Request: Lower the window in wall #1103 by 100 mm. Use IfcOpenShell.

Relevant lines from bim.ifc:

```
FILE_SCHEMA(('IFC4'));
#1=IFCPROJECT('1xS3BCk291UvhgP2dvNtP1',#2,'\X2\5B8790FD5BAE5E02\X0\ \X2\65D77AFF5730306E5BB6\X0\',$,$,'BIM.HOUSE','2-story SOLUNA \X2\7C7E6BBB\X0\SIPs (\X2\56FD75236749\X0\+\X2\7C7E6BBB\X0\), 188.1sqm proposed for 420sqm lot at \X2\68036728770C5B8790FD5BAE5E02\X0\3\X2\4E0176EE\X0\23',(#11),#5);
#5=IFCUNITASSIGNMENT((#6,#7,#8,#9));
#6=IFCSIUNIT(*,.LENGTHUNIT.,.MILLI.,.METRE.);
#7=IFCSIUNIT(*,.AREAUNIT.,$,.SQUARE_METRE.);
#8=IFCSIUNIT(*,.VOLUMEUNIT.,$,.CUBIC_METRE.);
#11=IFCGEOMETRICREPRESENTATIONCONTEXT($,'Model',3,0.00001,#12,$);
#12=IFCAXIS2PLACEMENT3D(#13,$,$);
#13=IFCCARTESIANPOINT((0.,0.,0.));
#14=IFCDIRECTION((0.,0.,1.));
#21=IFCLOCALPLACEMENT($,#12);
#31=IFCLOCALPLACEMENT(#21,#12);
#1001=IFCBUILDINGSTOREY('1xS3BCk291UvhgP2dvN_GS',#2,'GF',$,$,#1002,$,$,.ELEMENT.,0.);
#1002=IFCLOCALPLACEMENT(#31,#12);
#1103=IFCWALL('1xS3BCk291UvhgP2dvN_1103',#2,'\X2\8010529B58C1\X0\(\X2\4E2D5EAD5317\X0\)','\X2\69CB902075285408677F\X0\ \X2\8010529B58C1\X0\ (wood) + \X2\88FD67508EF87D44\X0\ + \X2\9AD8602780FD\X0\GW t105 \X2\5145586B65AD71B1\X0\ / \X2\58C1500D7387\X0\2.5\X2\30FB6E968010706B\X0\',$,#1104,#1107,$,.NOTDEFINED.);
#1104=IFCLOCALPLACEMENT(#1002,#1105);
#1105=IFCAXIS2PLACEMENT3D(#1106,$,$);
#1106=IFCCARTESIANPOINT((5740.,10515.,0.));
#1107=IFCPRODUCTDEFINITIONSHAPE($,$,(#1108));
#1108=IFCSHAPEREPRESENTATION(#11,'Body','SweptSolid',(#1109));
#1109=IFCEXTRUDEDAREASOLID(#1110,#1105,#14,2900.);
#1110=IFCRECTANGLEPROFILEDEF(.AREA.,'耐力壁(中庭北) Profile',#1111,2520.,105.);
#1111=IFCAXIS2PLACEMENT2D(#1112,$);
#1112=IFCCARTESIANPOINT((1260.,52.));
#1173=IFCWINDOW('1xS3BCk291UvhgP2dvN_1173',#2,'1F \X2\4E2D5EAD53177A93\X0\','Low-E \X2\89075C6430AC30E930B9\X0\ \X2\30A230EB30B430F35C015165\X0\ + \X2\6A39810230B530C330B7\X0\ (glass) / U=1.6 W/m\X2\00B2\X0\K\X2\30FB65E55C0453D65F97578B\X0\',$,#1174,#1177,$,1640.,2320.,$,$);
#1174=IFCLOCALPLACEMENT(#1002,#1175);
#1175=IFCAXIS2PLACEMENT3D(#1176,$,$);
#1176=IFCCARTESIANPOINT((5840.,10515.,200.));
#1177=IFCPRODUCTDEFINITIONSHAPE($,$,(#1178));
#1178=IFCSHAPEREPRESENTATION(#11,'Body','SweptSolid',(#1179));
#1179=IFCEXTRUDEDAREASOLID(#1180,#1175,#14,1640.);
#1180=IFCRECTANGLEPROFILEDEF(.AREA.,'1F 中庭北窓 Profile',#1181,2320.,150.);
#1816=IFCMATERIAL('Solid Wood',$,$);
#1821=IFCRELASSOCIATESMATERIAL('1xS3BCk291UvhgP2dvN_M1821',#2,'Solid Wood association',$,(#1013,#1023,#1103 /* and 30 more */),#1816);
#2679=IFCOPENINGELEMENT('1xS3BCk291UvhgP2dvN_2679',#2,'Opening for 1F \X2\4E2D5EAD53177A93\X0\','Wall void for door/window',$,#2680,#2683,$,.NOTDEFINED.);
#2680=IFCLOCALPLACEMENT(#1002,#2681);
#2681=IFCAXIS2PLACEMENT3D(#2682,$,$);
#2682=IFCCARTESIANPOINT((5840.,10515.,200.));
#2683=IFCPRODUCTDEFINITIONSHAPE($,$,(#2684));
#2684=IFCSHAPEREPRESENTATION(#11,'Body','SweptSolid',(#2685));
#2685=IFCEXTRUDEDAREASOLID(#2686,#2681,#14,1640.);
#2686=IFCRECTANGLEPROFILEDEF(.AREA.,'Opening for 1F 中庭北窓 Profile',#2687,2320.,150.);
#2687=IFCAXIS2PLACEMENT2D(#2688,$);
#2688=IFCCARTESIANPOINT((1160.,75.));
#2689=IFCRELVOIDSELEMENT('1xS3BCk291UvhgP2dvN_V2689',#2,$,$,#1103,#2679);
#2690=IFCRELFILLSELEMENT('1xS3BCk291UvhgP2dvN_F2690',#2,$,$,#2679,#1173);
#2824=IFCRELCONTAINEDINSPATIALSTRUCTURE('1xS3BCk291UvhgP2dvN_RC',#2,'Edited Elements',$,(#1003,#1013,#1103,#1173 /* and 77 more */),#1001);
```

```python
import numpy as np
import ifcopenshell
import ifcopenshell.api.geometry
import ifcopenshell.util.placement
import ifcopenshell.util.unit

model = ifcopenshell.open("bim.ifc")
unit_scale = ifcopenshell.util.unit.calculate_unit_scale(model)

window = model.by_guid("1xS3BCk291UvhgP2dvN_1173")
opening = window.FillsVoids[0].RelatingOpeningElement
dz = -0.1 / unit_scale

shift = np.array([0.0, 0.0, dz])
# The window is not placed relative to its opening, so move both.
for product in (opening, window):
    matrix = ifcopenshell.util.placement.get_local_placement(product.ObjectPlacement)
    matrix[:3, 3] += shift
    ifcopenshell.api.geometry.edit_object_placement(model, product=product, matrix=matrix, is_si=False)

print(f"moved by {dz * unit_scale:+.3f} m")

model.write("bim_updated.ifc")
```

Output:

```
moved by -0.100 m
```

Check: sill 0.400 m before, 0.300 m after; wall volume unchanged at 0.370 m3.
